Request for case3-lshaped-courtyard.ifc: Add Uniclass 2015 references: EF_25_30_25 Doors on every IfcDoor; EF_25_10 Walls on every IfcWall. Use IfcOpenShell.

First a look at what the model holds.

```python
import ifcopenshell

model = ifcopenshell.open("case3-lshaped-courtyard.ifc")
print(model.schema)
print("classifications:", [c.Name for c in model.by_type("IfcClassification")])
for ifc_class in ("IfcDoor", "IfcRoof", "IfcStair", "IfcWall", "IfcWindow"):
    print(ifc_class, len(model.by_type(ifc_class)))
```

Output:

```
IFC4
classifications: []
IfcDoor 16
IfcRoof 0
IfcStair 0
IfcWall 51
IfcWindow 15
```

```python
import ifcopenshell
import ifcopenshell.api.classification

model = ifcopenshell.open("case3-lshaped-courtyard.ifc")

system = ifcopenshell.api.classification.add_classification(model, classification="Uniclass 2015")

codes = {
    "IfcDoor": ("EF_25_30_25", "Doors"),
    "IfcWall": ("EF_25_10", "Walls"),
}
for ifc_class, (code, name) in codes.items():
    products = model.by_type(ifc_class)
    ifcopenshell.api.classification.add_reference(
        model, products=products, classification=system, identification=code, name=name
    )
    print(code, len(products))

model.write("case3-lshaped-courtyard_edited.ifc")
```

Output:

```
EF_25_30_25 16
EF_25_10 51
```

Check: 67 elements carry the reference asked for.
